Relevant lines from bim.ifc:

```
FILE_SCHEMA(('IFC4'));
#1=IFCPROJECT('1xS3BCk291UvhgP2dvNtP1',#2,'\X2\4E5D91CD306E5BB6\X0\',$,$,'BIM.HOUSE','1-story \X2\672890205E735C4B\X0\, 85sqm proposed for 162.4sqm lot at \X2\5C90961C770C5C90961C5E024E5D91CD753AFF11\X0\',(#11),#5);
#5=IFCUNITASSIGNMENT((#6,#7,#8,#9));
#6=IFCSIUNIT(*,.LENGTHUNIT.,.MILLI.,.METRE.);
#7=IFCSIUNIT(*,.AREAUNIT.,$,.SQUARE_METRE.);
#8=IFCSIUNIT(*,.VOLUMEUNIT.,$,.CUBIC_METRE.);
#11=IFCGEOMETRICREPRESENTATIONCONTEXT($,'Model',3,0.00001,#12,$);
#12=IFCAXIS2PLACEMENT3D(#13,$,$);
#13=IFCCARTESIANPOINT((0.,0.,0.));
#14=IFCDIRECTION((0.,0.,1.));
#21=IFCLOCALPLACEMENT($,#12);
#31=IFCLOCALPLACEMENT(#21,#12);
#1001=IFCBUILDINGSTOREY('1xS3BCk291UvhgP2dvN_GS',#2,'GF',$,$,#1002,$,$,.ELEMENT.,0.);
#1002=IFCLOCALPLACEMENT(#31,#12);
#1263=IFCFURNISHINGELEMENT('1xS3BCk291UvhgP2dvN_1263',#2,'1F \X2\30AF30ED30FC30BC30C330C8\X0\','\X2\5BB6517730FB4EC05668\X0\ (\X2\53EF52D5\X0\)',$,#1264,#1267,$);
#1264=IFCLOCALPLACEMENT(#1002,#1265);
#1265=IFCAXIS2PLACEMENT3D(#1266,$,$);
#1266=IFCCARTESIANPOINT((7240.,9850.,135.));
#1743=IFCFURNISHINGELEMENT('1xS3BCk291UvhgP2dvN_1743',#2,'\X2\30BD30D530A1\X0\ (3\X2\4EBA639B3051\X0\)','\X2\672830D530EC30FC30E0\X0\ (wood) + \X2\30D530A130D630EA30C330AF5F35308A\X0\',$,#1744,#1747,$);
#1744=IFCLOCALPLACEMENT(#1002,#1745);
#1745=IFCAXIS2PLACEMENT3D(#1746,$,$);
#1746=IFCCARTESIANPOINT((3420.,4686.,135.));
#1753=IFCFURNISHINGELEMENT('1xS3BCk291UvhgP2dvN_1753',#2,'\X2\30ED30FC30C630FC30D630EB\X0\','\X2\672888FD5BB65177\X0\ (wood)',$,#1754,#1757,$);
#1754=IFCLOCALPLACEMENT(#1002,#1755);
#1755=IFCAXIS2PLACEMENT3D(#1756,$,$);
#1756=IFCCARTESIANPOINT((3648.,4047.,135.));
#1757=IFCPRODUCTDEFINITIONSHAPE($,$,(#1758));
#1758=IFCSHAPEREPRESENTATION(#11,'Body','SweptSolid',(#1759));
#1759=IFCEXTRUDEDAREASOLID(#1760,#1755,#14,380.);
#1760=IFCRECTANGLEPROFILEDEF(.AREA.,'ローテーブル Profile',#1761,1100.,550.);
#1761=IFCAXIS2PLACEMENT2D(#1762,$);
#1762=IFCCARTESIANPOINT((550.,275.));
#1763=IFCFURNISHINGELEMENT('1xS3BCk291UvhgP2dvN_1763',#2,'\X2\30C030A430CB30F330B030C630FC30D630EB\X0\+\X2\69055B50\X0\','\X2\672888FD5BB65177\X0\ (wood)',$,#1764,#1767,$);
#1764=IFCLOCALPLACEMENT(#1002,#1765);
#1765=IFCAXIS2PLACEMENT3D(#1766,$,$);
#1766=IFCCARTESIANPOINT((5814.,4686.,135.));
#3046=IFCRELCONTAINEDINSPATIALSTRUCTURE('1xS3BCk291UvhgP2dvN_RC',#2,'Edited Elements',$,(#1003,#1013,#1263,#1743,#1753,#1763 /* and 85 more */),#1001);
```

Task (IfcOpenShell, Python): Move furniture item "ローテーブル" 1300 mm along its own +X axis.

```python
import ifcopenshell
import ifcopenshell.api.geometry
import ifcopenshell.util.placement
import ifcopenshell.util.unit

model = ifcopenshell.open("bim.ifc")
unit_scale = ifcopenshell.util.unit.calculate_unit_scale(model)

item = model.by_guid("1xS3BCk291UvhgP2dvN_1753")
matrix = ifcopenshell.util.placement.get_local_placement(item.ObjectPlacement)
matrix[:3, 3] += matrix[:3, 0] * 1.3 / unit_scale
ifcopenshell.api.geometry.edit_object_placement(model, product=item, matrix=matrix, is_si=False)

print(ifcopenshell.util.placement.get_local_placement(item.ObjectPlacement).round(3) + 0.0)

model.write("bim_updated.ifc")
```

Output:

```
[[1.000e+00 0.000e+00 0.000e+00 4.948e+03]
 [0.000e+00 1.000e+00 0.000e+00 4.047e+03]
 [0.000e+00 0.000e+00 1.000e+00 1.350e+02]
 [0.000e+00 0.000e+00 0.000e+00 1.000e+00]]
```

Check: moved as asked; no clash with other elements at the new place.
